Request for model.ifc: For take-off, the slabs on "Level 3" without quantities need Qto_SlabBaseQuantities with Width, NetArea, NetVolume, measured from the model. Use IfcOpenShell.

First a look at what the model holds.

```python
import ifcopenshell
import ifcopenshell.util.element
import ifcopenshell.util.unit

model = ifcopenshell.open("model.ifc")
print(model.schema)
for unit_type in ("LENGTHUNIT", "AREAUNIT", "VOLUMEUNIT"):
    print(unit_type, ifcopenshell.util.unit.calculate_unit_scale(model, unit_type))
storey = next(s for s in model.by_type("IfcBuildingStorey") if s.Name == "Level 3")
slabs = [e for e in ifcopenshell.util.element.get_decomposition(storey) if e.is_a("IfcSlab")]
for e in sorted(slabs, key=lambda e: e.id()):
    print(e.id(), e.is_a(), e.Name, list(ifcopenshell.util.element.get_psets(e, qtos_only=True)), sep=" | ")
```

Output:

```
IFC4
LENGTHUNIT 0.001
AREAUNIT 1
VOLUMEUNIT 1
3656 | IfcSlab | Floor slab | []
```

```python
import ifcopenshell
import ifcopenshell.api.pset
import ifcopenshell.geom
import ifcopenshell.util.element
import ifcopenshell.util.shape
import ifcopenshell.util.unit

model = ifcopenshell.open("model.ifc")
unit_scale = ifcopenshell.util.unit.calculate_unit_scale(model)
area_scale = ifcopenshell.util.unit.calculate_unit_scale(model, "AREAUNIT")
volume_scale = ifcopenshell.util.unit.calculate_unit_scale(model, "VOLUMEUNIT")
settings = ifcopenshell.geom.settings()

storey = next(s for s in model.by_type("IfcBuildingStorey") if s.Name == "Level 3")
slabs = [e for e in ifcopenshell.util.element.get_decomposition(storey) if e.is_a("IfcSlab")]

for e in sorted(slabs, key=lambda e: e.id()):
    if ifcopenshell.util.element.get_psets(e, qtos_only=True, should_inherit=False):
        continue
    # Geometry comes back in metres, in the element's own axes.
    shape = ifcopenshell.geom.create_shape(settings, e)
    values = {
        "Width": ifcopenshell.util.shape.get_z(shape.geometry) / unit_scale,
        "NetArea": ifcopenshell.util.shape.get_footprint_area(shape.geometry) / area_scale,
        "NetVolume": ifcopenshell.util.shape.get_volume(shape.geometry) / volume_scale,
    }
    qto = ifcopenshell.api.pset.add_qto(model, product=e, name="Qto_SlabBaseQuantities")
    ifcopenshell.api.pset.edit_qto(model, qto=qto, properties=values)
    print(e.id(), {k: round(v, 3) for k, v in values.items()})

model.write("model-out.ifc")
```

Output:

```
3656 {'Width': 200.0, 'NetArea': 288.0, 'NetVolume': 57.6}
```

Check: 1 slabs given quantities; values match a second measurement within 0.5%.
